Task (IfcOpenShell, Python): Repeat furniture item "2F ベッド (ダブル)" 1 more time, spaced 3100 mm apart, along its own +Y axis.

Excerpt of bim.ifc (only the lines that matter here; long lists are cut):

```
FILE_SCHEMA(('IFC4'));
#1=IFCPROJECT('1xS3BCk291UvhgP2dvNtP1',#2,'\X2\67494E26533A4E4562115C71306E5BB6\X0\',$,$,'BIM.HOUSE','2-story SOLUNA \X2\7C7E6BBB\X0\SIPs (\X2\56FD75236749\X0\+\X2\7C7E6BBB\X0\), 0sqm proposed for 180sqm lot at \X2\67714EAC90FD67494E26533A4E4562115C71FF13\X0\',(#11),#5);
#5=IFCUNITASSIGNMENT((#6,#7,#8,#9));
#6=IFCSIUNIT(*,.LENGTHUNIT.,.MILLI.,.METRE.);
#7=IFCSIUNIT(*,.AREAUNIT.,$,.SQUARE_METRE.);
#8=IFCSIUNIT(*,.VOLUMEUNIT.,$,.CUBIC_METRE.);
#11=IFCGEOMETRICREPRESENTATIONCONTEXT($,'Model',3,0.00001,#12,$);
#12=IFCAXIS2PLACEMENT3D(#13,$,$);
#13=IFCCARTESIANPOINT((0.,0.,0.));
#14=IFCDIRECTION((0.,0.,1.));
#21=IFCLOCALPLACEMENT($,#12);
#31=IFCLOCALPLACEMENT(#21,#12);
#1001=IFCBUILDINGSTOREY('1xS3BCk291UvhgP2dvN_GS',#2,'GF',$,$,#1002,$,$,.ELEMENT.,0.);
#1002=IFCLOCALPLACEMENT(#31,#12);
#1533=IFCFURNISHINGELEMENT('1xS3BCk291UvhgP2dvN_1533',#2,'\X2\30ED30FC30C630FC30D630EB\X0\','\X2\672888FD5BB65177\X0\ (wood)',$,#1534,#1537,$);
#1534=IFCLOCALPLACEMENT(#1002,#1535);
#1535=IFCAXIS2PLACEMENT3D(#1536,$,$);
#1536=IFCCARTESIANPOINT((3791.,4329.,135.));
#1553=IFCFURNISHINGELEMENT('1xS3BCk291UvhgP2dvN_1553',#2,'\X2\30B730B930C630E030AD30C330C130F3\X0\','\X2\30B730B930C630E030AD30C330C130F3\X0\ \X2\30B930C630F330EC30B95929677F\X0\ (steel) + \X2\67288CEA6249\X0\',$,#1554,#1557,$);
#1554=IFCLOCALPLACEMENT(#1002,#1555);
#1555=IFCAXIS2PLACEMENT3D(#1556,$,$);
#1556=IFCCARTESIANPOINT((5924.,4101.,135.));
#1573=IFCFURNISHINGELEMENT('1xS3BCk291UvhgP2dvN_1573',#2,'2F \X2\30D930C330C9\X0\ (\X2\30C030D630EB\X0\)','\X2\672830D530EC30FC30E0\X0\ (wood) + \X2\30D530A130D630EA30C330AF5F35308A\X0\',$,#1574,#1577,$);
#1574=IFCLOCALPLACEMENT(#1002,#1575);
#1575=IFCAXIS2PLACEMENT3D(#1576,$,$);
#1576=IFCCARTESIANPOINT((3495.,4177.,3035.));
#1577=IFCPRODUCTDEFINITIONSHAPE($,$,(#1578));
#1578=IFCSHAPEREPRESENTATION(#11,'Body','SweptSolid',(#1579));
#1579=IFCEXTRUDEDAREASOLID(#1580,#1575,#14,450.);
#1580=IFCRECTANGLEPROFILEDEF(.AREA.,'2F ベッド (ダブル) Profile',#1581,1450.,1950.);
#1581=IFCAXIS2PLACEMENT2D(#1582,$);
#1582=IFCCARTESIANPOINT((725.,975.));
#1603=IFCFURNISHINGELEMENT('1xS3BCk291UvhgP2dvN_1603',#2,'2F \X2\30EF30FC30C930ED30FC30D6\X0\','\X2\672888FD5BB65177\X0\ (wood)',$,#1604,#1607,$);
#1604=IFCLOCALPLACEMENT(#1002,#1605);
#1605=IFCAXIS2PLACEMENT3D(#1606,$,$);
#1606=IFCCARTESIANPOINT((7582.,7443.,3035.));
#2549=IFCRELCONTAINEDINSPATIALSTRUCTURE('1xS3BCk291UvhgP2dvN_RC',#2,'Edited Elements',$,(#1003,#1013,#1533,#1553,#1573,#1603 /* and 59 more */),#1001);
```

```python
import ifcopenshell
import ifcopenshell.api.geometry
import ifcopenshell.api.root
import ifcopenshell.util.element
import ifcopenshell.util.placement

model = ifcopenshell.open("bim.ifc")


def reuse_history(source, copy):
    """copy_class also copies each property set's owner history, people and application; keep the originals."""
    for rel in copy.IsDefinedBy:
        if rel.is_a("IfcRelDefinesByProperties") and (history := rel.RelatingPropertyDefinition.OwnerHistory):
            rel.RelatingPropertyDefinition.OwnerHistory = source.OwnerHistory
            ifcopenshell.util.element.remove_deep2(model, history)


source = model.by_id(1573)
base = ifcopenshell.util.placement.get_local_placement(source.ObjectPlacement)
step = base[:3, 1] * 3100.0

for i in range(1, 2):
    copy = ifcopenshell.api.root.copy_class(model, product=source)
    copy.Representation = ifcopenshell.util.element.copy_deep(
        model, source.Representation, exclude=["IfcGeometricRepresentationContext", "IfcRepresentationMap"]
    )
    reuse_history(source, copy)
    matrix = base.copy()
    matrix[:3, 3] += i * step
    print("added at", matrix[:3, 3].round(3) + 0.0)
    ifcopenshell.api.geometry.edit_object_placement(model, product=copy, matrix=matrix, is_si=False)

model.write("bim_v2.ifc")
```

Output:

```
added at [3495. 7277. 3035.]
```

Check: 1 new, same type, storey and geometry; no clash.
